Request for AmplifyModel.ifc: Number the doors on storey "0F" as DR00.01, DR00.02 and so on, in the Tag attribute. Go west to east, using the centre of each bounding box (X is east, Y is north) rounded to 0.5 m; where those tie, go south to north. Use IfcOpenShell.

First a look at what the model holds.

```python
import ifcopenshell
import ifcopenshell.util.element
import ifcopenshell.util.placement

model = ifcopenshell.open("AmplifyModel.ifc")
print(model.schema)
storey = next(s for s in model.by_type("IfcBuildingStorey") if s.Name == "0F")
doors = [e for e in ifcopenshell.util.element.get_decomposition(storey) if e.is_a("IfcDoor")]
for e in sorted(doors, key=lambda e: e.id()):
    origin = ifcopenshell.util.placement.get_local_placement(e.ObjectPlacement)[:3, 3]
    print(e.id(), e.Tag, e.Name, origin.round(2) + 0.0, sep=" | ")
```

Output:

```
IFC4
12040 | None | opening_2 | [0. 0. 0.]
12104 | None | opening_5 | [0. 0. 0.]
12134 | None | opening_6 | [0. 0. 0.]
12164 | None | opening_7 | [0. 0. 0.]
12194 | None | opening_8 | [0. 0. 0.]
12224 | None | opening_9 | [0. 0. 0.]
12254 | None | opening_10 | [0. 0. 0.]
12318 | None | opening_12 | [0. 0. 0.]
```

```python
import ifcopenshell
import ifcopenshell.geom
import ifcopenshell.util.element
import ifcopenshell.util.shape

model = ifcopenshell.open("AmplifyModel.ifc")
settings = ifcopenshell.geom.settings()
settings.set("use-world-coords", True)


def centre(element):
    shape = ifcopenshell.geom.create_shape(settings, element)
    return ifcopenshell.util.shape.get_bbox_centroid(shape.geometry)


storey = next(s for s in model.by_type("IfcBuildingStorey") if s.Name == "0F")
doors = [e for e in ifcopenshell.util.element.get_decomposition(storey) if e.is_a("IfcDoor")]

# Insertion points can sit at a corner or the storey origin, so sort by the geometry (in metres).
centres = {e: centre(e) for e in doors}
doors.sort(key=lambda e: (round(centres[e][0] / 0.5), centres[e][1]))

for i, e in enumerate(doors, start=1):
    number = f"DR00.{i:02d}"
    e.Tag = number
    print(e.id(), number)

model.write("AmplifyModel_v2.ifc")
```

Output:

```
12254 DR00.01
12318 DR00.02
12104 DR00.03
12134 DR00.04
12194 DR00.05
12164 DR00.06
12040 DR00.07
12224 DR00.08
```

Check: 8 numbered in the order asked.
